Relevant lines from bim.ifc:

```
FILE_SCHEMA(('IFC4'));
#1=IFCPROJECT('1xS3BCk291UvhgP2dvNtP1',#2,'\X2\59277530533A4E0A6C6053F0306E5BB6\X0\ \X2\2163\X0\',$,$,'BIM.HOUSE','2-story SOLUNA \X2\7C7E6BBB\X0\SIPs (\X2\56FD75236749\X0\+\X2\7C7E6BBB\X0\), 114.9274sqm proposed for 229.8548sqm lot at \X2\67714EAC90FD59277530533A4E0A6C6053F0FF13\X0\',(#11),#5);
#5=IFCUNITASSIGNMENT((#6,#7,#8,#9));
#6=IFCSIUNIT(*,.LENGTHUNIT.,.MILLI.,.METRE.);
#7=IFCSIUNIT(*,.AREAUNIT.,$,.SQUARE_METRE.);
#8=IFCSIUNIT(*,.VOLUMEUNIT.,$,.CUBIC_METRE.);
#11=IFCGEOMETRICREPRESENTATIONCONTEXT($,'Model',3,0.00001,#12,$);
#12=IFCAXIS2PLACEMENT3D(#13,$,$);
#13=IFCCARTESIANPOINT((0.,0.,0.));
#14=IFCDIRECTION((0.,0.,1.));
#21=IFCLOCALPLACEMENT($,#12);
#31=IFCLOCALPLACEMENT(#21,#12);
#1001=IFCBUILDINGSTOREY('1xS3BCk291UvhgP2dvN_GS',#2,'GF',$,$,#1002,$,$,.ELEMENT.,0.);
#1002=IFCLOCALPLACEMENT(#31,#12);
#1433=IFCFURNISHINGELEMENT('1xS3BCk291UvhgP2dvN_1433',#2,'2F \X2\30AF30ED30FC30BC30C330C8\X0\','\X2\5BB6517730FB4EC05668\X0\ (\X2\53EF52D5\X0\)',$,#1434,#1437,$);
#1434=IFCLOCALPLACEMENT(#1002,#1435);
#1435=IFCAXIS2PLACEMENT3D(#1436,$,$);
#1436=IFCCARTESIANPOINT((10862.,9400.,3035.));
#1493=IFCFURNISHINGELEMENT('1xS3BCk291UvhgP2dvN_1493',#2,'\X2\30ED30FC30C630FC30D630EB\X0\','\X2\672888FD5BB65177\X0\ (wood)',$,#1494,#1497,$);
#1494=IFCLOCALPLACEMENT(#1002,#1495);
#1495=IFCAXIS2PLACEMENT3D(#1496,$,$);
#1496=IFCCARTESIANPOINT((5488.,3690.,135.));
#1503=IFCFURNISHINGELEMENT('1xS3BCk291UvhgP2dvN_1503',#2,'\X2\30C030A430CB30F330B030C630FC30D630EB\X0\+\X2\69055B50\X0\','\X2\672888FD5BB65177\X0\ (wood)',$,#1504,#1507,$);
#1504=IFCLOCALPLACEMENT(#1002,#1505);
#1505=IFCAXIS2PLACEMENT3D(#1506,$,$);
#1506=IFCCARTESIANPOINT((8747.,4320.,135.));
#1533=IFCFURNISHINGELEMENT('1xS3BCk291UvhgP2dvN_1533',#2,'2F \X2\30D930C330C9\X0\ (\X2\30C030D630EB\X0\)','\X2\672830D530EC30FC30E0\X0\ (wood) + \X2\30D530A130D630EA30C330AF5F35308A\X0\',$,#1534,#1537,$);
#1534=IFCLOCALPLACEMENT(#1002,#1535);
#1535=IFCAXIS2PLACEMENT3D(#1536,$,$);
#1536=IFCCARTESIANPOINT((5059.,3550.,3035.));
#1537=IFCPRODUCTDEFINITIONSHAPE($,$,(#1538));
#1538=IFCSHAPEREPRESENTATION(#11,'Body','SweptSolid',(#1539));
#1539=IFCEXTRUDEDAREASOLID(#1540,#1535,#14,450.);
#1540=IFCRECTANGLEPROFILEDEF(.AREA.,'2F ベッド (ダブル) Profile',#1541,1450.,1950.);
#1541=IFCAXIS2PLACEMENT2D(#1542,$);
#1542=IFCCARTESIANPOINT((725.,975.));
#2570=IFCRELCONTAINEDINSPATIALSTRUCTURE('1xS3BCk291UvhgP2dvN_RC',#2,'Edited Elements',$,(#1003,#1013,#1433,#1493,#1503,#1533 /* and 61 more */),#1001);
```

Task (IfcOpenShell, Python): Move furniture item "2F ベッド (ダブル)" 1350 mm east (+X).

```python
import ifcopenshell
import ifcopenshell.api.geometry
import ifcopenshell.util.placement
import ifcopenshell.util.unit

model = ifcopenshell.open("bim.ifc")
unit_scale = ifcopenshell.util.unit.calculate_unit_scale(model)

item = model.by_guid("1xS3BCk291UvhgP2dvN_1533")
matrix = ifcopenshell.util.placement.get_local_placement(item.ObjectPlacement)
matrix[0, 3] += 1.35 / unit_scale
ifcopenshell.api.geometry.edit_object_placement(model, product=item, matrix=matrix, is_si=False)

print(ifcopenshell.util.placement.get_local_placement(item.ObjectPlacement).round(3) + 0.0)

model.write("bim-out.ifc")
```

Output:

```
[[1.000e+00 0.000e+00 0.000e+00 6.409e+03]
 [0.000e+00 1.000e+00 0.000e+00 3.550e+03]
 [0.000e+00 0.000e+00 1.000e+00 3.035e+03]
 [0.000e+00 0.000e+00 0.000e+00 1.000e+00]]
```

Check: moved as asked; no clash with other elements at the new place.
